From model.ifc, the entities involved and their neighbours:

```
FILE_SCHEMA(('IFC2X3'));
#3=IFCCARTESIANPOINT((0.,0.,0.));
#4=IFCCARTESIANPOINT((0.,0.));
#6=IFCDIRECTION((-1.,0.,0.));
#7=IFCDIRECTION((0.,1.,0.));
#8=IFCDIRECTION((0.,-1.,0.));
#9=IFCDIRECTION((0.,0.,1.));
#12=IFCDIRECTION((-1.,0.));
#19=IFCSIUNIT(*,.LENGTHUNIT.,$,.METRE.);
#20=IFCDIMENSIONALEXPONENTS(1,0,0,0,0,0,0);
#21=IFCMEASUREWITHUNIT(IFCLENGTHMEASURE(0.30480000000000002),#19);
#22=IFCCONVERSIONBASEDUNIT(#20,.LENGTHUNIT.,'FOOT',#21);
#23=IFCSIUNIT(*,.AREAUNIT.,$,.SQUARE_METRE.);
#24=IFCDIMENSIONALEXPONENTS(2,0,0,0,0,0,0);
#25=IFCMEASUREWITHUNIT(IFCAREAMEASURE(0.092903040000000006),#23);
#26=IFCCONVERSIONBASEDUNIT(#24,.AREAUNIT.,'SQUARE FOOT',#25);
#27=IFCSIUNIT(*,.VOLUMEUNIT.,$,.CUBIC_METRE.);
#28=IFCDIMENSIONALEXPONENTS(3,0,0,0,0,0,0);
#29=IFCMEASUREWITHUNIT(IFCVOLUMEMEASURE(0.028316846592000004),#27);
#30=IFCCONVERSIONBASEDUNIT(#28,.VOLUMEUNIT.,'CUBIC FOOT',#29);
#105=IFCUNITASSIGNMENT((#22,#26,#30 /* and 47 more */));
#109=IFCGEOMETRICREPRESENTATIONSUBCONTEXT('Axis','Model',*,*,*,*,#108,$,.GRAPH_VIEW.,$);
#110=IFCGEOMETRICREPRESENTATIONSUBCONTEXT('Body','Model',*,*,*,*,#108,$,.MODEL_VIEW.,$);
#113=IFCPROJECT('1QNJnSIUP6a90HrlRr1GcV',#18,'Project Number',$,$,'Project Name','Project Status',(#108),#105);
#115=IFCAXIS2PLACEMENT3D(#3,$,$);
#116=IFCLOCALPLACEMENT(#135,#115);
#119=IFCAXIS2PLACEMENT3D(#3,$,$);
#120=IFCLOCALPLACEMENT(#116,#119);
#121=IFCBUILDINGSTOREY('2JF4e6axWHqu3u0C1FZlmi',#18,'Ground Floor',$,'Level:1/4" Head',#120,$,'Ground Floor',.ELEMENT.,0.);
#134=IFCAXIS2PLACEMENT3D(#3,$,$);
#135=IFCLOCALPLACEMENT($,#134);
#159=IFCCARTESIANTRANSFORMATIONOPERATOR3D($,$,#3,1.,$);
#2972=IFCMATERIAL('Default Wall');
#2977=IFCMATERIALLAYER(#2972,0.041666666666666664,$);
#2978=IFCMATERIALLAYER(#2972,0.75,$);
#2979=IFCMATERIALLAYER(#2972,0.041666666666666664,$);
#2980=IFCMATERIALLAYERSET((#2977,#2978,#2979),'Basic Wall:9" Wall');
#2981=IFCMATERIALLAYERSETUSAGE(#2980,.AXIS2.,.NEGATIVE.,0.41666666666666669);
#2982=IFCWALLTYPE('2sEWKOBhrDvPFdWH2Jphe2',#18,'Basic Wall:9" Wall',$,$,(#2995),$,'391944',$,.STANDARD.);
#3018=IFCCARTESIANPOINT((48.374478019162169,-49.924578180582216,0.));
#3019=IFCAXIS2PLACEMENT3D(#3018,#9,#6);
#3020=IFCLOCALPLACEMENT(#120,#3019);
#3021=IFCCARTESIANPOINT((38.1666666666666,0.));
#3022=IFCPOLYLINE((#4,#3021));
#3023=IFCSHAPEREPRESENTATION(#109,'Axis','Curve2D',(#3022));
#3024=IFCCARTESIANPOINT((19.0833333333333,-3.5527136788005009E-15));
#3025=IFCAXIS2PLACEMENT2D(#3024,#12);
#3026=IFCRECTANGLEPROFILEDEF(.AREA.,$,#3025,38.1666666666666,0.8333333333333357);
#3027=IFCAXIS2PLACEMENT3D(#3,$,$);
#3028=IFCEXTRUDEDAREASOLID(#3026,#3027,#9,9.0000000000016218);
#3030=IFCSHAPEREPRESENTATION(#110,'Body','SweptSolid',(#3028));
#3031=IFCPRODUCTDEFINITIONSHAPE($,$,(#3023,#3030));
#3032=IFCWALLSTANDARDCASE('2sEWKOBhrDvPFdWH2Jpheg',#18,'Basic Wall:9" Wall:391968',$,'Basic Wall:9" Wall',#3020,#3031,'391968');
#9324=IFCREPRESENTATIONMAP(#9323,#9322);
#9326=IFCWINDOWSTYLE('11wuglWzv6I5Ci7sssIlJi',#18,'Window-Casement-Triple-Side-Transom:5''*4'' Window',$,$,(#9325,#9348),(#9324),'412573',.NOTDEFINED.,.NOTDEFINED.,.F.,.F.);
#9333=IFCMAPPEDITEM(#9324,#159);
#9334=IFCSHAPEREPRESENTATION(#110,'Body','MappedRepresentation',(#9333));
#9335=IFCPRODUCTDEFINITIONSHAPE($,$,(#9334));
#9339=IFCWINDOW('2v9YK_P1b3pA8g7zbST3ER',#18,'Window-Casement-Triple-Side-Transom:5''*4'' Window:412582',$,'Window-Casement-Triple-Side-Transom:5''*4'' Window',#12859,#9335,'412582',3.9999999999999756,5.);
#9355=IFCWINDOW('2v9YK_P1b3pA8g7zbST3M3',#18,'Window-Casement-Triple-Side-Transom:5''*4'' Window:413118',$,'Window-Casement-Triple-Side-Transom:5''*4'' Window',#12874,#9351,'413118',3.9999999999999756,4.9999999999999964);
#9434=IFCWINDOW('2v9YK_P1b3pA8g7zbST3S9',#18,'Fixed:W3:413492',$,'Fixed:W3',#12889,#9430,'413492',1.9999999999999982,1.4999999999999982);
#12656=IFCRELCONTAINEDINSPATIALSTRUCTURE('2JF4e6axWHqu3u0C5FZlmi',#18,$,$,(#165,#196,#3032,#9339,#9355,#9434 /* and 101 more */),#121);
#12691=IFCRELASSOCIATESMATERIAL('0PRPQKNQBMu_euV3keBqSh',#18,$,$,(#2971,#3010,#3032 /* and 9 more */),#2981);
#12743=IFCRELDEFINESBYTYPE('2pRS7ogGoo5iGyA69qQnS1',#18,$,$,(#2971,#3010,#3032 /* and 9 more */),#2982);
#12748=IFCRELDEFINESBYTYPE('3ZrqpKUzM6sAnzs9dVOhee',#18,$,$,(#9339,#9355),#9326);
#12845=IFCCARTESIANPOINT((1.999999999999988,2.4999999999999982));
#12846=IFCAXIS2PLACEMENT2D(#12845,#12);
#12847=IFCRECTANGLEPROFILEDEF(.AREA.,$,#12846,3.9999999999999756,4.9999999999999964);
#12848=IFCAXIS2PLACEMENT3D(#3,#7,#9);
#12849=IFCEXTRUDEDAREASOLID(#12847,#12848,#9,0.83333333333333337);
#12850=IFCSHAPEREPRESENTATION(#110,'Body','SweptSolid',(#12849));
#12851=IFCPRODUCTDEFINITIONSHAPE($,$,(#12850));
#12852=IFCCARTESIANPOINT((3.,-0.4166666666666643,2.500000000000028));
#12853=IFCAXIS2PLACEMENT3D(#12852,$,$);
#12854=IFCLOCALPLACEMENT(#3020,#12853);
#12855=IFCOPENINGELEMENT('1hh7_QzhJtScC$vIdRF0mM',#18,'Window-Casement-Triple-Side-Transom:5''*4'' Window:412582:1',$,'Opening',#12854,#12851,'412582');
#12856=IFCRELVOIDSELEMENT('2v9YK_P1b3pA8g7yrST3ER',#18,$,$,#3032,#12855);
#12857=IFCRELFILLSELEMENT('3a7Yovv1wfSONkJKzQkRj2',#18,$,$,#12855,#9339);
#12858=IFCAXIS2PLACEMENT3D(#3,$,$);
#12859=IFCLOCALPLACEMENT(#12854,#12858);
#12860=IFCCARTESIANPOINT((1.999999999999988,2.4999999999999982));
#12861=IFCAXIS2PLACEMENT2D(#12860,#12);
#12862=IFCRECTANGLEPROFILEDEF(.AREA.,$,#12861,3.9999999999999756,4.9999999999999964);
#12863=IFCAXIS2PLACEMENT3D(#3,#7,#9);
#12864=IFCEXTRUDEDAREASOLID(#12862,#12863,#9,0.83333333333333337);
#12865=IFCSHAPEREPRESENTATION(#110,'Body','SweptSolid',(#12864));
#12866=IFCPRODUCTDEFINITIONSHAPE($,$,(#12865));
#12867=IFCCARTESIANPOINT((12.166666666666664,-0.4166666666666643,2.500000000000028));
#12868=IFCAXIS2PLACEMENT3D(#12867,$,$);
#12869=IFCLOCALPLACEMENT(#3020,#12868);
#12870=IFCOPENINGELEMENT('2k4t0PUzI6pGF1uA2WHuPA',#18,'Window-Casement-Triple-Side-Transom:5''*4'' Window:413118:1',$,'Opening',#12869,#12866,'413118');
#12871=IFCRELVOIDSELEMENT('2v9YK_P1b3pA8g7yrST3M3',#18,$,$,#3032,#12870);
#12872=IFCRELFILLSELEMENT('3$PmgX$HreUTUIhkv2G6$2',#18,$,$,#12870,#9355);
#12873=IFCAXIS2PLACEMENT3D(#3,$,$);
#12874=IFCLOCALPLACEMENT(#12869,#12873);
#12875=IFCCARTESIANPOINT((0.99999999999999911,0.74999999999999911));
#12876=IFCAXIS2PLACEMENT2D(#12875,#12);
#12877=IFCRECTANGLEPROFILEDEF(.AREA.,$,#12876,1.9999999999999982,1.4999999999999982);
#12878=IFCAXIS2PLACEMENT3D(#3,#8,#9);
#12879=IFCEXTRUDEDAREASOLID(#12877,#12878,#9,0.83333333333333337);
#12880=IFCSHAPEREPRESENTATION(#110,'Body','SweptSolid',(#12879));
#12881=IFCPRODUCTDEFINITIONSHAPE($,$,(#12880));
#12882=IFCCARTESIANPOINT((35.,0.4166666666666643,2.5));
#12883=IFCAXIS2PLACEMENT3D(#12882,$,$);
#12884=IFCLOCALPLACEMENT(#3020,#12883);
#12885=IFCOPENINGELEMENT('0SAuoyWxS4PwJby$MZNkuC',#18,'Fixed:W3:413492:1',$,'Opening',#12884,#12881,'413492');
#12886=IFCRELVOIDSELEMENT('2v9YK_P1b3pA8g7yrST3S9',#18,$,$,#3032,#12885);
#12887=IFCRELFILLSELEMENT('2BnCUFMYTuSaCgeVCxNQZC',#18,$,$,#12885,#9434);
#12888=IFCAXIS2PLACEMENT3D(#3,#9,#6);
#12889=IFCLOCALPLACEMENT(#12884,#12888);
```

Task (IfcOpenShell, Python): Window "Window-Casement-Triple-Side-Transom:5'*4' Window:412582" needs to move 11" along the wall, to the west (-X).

```python
import ifcopenshell
import ifcopenshell.api.geometry
import ifcopenshell.util.placement
import ifcopenshell.util.unit

model = ifcopenshell.open("model.ifc")
unit_scale = ifcopenshell.util.unit.calculate_unit_scale(model)

window = model.by_guid("2v9YK_P1b3pA8g7zbST3ER")
opening = window.FillsVoids[0].RelatingOpeningElement
wall = opening.VoidsElements[0].RelatingBuildingElement

wall_matrix = ifcopenshell.util.placement.get_local_placement(wall.ObjectPlacement)
shift = wall_matrix[:3, 0] * 11 * 0.0254 / unit_scale
before = ifcopenshell.util.placement.get_local_placement(window.ObjectPlacement)[:3, 3].copy()

# The window is placed relative to its opening, so it follows when the opening moves.
matrix = ifcopenshell.util.placement.get_local_placement(opening.ObjectPlacement)
matrix[:3, 3] += shift
ifcopenshell.api.geometry.edit_object_placement(
    model, product=opening, matrix=matrix, is_si=False, should_transform_children=True
)

after = ifcopenshell.util.placement.get_local_placement(window.ObjectPlacement)[:3, 3]
print("window moved by", (after - before).round(3) + 0.0)

model.write("model_v2.ifc")
```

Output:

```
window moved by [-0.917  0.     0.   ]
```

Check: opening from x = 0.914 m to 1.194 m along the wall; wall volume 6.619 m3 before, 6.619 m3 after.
